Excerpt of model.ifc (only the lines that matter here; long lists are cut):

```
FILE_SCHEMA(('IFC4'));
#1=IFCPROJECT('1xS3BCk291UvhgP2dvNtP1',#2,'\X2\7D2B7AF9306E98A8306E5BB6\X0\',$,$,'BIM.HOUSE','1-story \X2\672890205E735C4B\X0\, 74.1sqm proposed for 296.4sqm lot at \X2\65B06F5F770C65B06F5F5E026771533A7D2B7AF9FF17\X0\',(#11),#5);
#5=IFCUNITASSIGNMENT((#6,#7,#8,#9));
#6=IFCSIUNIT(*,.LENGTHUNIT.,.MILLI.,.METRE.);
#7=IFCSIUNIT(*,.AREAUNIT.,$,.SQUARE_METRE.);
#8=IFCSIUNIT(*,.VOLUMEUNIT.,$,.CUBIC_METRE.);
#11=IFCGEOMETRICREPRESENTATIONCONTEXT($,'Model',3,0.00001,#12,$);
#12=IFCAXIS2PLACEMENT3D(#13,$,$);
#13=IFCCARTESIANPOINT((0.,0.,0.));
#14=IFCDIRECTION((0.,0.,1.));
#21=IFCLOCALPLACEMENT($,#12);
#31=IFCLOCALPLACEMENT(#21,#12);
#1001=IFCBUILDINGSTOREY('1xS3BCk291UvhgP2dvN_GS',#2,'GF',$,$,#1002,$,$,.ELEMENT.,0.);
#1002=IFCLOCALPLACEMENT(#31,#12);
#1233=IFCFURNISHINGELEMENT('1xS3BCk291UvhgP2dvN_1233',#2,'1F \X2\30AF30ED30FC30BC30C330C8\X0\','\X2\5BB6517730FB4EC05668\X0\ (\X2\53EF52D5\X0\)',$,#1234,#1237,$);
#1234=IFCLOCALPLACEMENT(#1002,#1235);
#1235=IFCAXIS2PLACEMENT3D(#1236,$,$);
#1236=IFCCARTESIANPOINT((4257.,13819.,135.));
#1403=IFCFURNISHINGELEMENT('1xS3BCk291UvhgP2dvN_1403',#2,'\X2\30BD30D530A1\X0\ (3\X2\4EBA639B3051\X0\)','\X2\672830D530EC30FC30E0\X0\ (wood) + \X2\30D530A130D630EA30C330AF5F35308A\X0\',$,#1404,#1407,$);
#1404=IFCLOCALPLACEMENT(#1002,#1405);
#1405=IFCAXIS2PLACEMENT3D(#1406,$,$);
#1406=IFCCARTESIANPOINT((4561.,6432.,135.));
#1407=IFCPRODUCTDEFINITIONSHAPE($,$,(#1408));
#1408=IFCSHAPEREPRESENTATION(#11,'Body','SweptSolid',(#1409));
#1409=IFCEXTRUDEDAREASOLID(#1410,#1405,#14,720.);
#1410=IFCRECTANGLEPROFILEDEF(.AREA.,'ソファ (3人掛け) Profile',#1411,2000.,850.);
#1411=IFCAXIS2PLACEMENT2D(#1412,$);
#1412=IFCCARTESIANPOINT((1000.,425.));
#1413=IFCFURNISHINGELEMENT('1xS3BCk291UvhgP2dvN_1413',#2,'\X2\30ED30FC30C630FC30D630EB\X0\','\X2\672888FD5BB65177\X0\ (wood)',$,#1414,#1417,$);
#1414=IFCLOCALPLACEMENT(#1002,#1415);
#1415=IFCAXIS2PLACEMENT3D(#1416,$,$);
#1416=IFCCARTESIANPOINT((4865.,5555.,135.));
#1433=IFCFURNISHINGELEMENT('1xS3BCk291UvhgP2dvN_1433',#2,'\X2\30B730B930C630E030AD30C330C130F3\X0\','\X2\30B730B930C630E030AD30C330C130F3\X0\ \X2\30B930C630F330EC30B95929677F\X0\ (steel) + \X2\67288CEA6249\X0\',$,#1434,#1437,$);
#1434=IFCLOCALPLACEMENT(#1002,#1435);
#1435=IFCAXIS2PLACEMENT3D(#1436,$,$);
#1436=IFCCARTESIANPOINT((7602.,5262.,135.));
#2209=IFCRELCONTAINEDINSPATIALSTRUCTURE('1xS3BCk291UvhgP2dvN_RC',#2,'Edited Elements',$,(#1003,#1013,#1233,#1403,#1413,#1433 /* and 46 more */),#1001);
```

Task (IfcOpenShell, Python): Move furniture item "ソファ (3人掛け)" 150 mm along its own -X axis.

```python
import ifcopenshell
import ifcopenshell.api.geometry
import ifcopenshell.util.placement

model = ifcopenshell.open("model.ifc")

item = model.by_id(1403)
matrix = ifcopenshell.util.placement.get_local_placement(item.ObjectPlacement)
matrix[:3, 3] -= matrix[:3, 0] * 150.0
ifcopenshell.api.geometry.edit_object_placement(model, product=item, matrix=matrix, is_si=False)

print(ifcopenshell.util.placement.get_local_placement(item.ObjectPlacement).round(3) + 0.0)

model.write("model_v2.ifc")
```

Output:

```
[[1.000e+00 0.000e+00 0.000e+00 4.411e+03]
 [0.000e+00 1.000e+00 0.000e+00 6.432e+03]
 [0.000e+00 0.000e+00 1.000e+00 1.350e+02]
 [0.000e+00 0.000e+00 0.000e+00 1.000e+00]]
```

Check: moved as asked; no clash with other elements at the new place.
